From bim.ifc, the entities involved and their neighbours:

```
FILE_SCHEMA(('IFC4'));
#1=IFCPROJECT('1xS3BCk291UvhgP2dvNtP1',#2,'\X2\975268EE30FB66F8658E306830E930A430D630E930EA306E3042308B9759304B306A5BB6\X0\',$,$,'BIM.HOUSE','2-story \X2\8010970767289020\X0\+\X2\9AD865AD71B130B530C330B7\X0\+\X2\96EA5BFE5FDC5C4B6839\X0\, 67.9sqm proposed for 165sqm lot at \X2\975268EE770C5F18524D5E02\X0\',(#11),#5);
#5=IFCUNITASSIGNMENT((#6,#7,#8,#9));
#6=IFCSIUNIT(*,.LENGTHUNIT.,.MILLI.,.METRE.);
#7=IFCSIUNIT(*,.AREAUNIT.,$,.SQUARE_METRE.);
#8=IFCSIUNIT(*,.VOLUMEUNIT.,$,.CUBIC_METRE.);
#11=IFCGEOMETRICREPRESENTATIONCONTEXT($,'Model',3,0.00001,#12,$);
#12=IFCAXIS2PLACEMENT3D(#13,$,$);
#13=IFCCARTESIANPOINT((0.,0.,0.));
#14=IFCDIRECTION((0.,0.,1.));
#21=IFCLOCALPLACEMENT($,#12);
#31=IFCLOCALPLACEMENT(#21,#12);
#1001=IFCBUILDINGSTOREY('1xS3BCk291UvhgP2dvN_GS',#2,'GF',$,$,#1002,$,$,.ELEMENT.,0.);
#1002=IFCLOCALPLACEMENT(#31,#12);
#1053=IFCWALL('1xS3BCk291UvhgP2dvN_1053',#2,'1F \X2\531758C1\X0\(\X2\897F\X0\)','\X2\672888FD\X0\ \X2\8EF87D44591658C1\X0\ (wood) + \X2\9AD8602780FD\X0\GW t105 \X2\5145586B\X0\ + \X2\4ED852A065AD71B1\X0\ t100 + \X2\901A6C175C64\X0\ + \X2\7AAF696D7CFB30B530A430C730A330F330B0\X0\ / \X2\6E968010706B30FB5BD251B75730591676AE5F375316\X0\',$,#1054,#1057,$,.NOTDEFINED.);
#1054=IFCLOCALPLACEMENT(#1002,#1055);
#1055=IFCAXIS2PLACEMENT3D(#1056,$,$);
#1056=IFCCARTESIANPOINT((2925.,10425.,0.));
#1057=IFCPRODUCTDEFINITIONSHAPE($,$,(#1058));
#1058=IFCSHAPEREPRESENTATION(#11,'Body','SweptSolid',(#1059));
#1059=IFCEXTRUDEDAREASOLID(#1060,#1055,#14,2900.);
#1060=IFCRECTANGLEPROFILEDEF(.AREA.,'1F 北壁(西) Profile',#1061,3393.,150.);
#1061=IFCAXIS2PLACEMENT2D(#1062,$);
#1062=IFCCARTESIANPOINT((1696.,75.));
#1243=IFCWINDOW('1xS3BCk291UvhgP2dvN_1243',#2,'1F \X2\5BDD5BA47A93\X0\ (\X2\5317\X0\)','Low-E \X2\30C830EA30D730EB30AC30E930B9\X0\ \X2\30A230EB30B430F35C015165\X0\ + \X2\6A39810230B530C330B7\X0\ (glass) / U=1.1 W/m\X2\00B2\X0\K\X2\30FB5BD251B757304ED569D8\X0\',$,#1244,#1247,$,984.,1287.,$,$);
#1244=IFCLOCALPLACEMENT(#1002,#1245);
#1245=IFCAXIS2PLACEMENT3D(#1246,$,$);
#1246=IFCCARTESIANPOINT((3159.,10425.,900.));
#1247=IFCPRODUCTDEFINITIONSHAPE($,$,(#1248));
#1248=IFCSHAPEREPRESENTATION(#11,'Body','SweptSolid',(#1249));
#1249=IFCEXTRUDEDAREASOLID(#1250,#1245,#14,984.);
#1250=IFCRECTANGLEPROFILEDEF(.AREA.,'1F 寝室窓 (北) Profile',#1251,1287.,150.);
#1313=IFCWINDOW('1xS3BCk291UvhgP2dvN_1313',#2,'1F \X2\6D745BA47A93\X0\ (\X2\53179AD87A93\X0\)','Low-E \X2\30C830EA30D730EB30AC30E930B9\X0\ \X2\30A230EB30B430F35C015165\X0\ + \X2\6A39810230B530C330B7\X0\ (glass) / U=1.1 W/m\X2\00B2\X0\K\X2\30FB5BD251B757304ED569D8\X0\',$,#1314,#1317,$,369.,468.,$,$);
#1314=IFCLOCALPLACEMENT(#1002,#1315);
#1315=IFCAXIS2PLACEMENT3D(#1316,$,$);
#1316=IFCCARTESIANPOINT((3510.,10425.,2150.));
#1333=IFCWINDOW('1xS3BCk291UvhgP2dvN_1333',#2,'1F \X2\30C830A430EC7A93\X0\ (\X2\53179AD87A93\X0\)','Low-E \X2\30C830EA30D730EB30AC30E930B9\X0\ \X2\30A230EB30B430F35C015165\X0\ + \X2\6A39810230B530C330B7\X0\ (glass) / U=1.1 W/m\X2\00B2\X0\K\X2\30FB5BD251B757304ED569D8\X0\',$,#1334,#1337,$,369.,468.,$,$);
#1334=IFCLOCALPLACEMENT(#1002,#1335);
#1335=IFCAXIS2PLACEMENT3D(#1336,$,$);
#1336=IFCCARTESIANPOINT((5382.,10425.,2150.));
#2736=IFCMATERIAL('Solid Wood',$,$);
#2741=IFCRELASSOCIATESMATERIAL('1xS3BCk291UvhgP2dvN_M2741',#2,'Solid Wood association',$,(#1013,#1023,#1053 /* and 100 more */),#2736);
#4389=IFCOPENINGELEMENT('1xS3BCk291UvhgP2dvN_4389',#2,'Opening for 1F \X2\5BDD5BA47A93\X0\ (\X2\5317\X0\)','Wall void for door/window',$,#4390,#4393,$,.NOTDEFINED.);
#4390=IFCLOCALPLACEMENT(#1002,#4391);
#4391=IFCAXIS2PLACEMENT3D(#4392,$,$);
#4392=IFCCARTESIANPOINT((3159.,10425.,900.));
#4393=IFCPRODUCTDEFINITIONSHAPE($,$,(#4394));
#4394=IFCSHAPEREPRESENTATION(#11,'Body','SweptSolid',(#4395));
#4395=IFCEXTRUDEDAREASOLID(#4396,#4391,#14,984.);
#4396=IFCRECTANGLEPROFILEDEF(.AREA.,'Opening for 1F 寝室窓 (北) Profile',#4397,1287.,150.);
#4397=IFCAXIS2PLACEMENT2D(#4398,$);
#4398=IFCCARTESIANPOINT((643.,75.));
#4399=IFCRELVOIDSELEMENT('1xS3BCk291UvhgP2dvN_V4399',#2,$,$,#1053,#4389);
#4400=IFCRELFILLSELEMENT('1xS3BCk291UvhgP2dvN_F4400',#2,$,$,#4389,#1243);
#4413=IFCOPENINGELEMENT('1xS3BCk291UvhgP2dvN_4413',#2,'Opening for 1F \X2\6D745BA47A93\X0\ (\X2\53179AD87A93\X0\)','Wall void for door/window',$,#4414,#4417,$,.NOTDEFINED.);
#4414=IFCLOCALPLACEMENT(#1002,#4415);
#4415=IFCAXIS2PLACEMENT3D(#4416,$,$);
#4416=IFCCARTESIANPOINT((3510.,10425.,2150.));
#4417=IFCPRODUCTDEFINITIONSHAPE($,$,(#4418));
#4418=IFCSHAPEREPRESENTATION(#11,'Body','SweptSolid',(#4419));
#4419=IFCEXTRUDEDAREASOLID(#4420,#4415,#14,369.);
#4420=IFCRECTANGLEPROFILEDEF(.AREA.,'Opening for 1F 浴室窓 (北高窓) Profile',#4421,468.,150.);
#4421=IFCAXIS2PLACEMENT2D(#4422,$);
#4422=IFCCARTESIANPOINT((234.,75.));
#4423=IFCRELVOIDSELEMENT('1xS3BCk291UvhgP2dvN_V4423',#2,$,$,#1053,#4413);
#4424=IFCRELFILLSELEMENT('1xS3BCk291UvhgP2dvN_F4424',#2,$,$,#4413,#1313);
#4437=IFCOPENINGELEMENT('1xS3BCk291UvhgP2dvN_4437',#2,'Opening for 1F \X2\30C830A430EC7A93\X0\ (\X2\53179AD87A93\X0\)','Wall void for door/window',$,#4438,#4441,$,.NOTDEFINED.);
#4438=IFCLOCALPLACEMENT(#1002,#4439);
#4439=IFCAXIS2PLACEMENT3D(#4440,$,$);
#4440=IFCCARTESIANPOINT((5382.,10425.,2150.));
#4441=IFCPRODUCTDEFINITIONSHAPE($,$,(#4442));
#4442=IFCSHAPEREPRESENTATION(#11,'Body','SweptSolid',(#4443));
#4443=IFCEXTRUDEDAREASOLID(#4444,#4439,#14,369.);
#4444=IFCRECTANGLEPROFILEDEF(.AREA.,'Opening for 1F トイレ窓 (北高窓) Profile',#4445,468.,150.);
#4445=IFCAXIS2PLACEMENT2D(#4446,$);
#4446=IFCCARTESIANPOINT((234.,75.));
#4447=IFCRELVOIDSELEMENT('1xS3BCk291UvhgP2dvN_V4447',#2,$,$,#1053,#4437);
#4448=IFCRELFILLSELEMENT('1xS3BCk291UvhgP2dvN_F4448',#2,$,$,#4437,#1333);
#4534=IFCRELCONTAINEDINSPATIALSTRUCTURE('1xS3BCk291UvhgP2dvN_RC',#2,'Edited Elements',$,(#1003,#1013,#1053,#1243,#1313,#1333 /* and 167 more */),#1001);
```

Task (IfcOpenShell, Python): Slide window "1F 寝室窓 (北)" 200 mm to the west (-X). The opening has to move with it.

```python
import ifcopenshell
import ifcopenshell.api.geometry
import ifcopenshell.util.placement
import ifcopenshell.util.unit

model = ifcopenshell.open("bim.ifc")
unit_scale = ifcopenshell.util.unit.calculate_unit_scale(model)

window = model.by_id(1243)
opening = window.FillsVoids[0].RelatingOpeningElement
wall = opening.VoidsElements[0].RelatingBuildingElement

wall_matrix = ifcopenshell.util.placement.get_local_placement(wall.ObjectPlacement)
shift = wall_matrix[:3, 0] * -0.2 / unit_scale
before = ifcopenshell.util.placement.get_local_placement(window.ObjectPlacement)[:3, 3].copy()

# The window is not placed relative to its opening, so move both.
for product in (opening, window):
    matrix = ifcopenshell.util.placement.get_local_placement(product.ObjectPlacement)
    matrix[:3, 3] += shift
    ifcopenshell.api.geometry.edit_object_placement(model, product=product, matrix=matrix, is_si=False)

after = ifcopenshell.util.placement.get_local_placement(window.ObjectPlacement)[:3, 3]
print("window moved by", (after - before).round(3) + 0.0)

model.write("bim_rev.ifc")
```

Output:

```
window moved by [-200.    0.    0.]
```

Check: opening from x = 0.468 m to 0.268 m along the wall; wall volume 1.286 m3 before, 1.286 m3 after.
